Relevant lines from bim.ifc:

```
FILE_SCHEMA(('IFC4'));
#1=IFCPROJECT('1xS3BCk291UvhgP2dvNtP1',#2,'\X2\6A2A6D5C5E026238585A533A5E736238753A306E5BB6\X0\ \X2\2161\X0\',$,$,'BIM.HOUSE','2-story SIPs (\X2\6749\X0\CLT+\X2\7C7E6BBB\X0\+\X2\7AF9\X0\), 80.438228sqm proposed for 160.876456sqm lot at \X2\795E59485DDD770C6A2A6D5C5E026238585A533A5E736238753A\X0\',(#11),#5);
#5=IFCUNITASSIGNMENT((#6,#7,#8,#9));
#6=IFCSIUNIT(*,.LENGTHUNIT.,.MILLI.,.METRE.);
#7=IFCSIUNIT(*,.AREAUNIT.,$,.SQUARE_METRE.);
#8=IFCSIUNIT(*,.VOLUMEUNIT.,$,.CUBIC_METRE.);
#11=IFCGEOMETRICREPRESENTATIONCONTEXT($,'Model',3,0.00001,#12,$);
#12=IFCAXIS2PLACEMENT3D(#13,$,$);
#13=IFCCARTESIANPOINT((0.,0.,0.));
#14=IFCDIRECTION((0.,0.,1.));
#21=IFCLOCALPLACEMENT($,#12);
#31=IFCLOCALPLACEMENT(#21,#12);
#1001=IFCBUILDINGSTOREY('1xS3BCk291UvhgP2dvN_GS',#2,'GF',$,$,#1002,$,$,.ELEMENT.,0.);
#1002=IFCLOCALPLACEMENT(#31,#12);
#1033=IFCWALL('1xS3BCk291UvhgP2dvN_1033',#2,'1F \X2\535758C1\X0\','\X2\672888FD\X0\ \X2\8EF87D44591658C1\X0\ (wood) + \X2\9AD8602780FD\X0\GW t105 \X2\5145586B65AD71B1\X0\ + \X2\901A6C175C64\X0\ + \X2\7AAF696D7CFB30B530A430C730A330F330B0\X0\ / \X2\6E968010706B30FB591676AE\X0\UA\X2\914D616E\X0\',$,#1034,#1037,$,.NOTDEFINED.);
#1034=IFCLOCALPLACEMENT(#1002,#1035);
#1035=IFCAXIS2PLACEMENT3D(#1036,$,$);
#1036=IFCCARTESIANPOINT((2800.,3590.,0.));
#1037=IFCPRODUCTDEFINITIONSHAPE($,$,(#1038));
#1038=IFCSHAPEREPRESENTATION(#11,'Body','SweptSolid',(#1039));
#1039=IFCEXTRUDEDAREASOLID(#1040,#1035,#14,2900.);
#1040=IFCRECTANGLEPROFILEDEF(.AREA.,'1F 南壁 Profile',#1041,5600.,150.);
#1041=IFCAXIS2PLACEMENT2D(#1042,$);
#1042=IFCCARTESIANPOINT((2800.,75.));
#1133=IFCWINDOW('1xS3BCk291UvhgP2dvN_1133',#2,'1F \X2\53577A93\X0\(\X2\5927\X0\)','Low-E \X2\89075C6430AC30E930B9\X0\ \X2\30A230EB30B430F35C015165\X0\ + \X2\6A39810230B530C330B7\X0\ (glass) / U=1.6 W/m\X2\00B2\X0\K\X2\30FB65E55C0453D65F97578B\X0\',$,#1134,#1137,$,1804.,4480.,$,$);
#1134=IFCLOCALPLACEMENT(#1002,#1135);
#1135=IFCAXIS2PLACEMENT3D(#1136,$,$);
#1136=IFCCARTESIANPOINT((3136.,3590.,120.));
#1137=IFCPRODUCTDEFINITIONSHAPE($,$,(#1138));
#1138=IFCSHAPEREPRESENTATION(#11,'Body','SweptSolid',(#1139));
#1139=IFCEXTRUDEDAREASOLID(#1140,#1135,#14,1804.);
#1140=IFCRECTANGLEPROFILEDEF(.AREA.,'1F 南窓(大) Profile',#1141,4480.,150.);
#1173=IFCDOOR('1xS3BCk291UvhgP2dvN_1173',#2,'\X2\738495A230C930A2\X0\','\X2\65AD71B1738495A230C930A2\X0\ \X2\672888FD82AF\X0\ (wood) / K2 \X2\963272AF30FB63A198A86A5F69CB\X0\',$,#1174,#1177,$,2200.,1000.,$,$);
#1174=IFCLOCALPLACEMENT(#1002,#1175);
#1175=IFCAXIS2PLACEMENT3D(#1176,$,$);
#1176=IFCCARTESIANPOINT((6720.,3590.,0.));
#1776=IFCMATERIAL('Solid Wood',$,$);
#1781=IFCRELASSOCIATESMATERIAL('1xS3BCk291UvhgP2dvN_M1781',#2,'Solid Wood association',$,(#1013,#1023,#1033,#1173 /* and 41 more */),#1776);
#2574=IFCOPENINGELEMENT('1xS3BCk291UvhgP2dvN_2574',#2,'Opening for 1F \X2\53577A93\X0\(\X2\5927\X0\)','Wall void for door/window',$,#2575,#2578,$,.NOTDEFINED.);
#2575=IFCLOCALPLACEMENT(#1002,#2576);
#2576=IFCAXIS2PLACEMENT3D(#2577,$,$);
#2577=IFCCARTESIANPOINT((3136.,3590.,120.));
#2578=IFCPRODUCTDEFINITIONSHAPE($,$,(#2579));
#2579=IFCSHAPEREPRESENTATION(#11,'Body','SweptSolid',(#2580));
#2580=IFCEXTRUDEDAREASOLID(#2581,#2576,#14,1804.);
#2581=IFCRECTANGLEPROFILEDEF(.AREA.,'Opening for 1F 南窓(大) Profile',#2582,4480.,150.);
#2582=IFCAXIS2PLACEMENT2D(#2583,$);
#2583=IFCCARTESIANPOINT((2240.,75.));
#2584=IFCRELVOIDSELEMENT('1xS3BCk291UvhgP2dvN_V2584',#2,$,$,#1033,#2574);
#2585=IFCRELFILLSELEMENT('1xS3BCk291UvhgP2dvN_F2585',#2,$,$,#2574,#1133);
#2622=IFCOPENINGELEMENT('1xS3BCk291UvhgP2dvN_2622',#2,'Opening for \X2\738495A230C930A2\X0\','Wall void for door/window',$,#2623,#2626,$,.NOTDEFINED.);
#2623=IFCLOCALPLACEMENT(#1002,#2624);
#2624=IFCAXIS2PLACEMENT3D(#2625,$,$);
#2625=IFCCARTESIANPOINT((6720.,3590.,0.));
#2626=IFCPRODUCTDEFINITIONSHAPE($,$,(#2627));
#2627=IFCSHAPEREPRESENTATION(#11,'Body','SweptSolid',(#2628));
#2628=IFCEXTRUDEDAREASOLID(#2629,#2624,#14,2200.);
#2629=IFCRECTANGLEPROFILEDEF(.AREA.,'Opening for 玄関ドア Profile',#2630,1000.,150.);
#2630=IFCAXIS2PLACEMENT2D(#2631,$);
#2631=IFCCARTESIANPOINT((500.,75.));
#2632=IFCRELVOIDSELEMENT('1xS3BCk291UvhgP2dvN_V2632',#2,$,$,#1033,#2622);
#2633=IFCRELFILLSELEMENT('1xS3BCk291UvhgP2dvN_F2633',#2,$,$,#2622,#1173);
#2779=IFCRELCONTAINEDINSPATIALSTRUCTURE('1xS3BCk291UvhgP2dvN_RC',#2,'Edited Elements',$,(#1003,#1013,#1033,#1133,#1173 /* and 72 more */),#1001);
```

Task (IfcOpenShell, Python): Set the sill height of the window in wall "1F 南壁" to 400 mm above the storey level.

```python
import numpy as np
import ifcopenshell
import ifcopenshell.api.geometry
import ifcopenshell.geom
import ifcopenshell.util.element
import ifcopenshell.util.placement
import ifcopenshell.util.shape
import ifcopenshell.util.unit

model = ifcopenshell.open("bim.ifc")
unit_scale = ifcopenshell.util.unit.calculate_unit_scale(model)

window = model.by_id(1133)
opening = window.FillsVoids[0].RelatingOpeningElement
storey = ifcopenshell.util.element.get_container(window, ifc_class="IfcBuildingStorey")
level = ifcopenshell.util.placement.get_local_placement(storey.ObjectPlacement)[2, 3]

# The opening's origin need not be at the sill, so measure its lowest point.
shape = ifcopenshell.geom.create_shape(ifcopenshell.geom.settings(), opening)
bottom = ifcopenshell.util.shape.get_shape_bottom_elevation(shape, shape.geometry) / unit_scale
dz = level + 400.0 - bottom

shift = np.array([0.0, 0.0, dz])
# The window is not placed relative to its opening, so move both.
for product in (opening, window):
    matrix = ifcopenshell.util.placement.get_local_placement(product.ObjectPlacement)
    matrix[:3, 3] += shift
    ifcopenshell.api.geometry.edit_object_placement(model, product=product, matrix=matrix, is_si=False)

print(f"moved by {dz * unit_scale:+.3f} m")

model.write("bim_updated.ifc")
```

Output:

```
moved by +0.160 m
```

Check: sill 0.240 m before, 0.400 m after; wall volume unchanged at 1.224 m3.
